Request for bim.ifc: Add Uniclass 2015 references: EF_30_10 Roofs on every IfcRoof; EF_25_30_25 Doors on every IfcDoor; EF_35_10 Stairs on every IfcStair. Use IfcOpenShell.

First a look at what the model holds.

```python
import ifcopenshell

model = ifcopenshell.open("bim.ifc")
print(model.schema)
print("classifications:", [c.Name for c in model.by_type("IfcClassification")])
for ifc_class in ("IfcDoor", "IfcRoof", "IfcStair", "IfcWall", "IfcWindow"):
    print(ifc_class, len(model.by_type(ifc_class)))
```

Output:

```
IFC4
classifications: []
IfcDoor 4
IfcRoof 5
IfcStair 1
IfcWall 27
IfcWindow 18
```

```python
import ifcopenshell
import ifcopenshell.api.classification

model = ifcopenshell.open("bim.ifc")

system = ifcopenshell.api.classification.add_classification(model, classification="Uniclass 2015")

codes = {
    "IfcRoof": ("EF_30_10", "Roofs"),
    "IfcDoor": ("EF_25_30_25", "Doors"),
    "IfcStair": ("EF_35_10", "Stairs"),
}
for ifc_class, (code, name) in codes.items():
    products = model.by_type(ifc_class)
    ifcopenshell.api.classification.add_reference(
        model, products=products, classification=system, identification=code, name=name
    )
    print(code, len(products))

model.write("bim-out.ifc")
```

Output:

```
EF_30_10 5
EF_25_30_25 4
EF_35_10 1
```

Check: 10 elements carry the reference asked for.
